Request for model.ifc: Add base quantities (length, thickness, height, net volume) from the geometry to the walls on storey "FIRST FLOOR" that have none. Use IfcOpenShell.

First a look at what the model holds.

```python
import ifcopenshell
import ifcopenshell.util.element
import ifcopenshell.util.unit

model = ifcopenshell.open("model.ifc")
print(model.schema)
for unit_type in ("LENGTHUNIT", "AREAUNIT", "VOLUMEUNIT"):
    print(unit_type, ifcopenshell.util.unit.calculate_unit_scale(model, unit_type))
storey = next(s for s in model.by_type("IfcBuildingStorey") if s.Name == "FIRST FLOOR")
walls = [e for e in ifcopenshell.util.element.get_decomposition(storey) if e.is_a("IfcWall")]
for e in sorted(walls, key=lambda e: e.id()):
    print(e.id(), e.is_a(), e.Name, list(ifcopenshell.util.element.get_psets(e, qtos_only=True)), sep=" | ")
```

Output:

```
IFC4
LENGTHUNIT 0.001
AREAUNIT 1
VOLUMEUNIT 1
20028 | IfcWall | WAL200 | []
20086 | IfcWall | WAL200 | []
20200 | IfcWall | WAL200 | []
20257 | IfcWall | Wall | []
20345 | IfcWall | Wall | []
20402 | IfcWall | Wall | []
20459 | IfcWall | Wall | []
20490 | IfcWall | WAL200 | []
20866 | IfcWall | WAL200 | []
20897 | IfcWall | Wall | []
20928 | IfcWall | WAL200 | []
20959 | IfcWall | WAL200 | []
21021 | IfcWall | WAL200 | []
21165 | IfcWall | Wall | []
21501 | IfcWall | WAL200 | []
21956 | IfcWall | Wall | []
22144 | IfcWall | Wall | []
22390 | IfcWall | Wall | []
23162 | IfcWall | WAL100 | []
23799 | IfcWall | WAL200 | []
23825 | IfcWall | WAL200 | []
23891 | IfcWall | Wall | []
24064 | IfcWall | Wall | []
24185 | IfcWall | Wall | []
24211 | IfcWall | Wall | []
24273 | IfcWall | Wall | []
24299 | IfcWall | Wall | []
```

```python
import ifcopenshell
import ifcopenshell.api.pset
import ifcopenshell.geom
import ifcopenshell.util.element
import ifcopenshell.util.shape
import ifcopenshell.util.unit

model = ifcopenshell.open("model.ifc")
unit_scale = ifcopenshell.util.unit.calculate_unit_scale(model)
volume_scale = ifcopenshell.util.unit.calculate_unit_scale(model, "VOLUMEUNIT")
settings = ifcopenshell.geom.settings()

storey = next(s for s in model.by_type("IfcBuildingStorey") if s.Name == "FIRST FLOOR")
walls = [e for e in ifcopenshell.util.element.get_decomposition(storey) if e.is_a("IfcWall")]

for e in sorted(walls, key=lambda e: e.id()):
    if ifcopenshell.util.element.get_psets(e, qtos_only=True, should_inherit=False):
        continue
    # Geometry comes back in metres, in the element's own axes.
    shape = ifcopenshell.geom.create_shape(settings, e)
    values = {
        "Length": ifcopenshell.util.shape.get_x(shape.geometry) / unit_scale,
        "Width": ifcopenshell.util.shape.get_y(shape.geometry) / unit_scale,
        "Height": ifcopenshell.util.shape.get_z(shape.geometry) / unit_scale,
        "NetVolume": ifcopenshell.util.shape.get_volume(shape.geometry) / volume_scale,
    }
    qto = ifcopenshell.api.pset.add_qto(model, product=e, name="Qto_WallBaseQuantities")
    ifcopenshell.api.pset.edit_qto(model, qto=qto, properties=values)
    print(e.id(), {k: round(v, 3) for k, v in values.items()})

model.write("model-out.ifc")
```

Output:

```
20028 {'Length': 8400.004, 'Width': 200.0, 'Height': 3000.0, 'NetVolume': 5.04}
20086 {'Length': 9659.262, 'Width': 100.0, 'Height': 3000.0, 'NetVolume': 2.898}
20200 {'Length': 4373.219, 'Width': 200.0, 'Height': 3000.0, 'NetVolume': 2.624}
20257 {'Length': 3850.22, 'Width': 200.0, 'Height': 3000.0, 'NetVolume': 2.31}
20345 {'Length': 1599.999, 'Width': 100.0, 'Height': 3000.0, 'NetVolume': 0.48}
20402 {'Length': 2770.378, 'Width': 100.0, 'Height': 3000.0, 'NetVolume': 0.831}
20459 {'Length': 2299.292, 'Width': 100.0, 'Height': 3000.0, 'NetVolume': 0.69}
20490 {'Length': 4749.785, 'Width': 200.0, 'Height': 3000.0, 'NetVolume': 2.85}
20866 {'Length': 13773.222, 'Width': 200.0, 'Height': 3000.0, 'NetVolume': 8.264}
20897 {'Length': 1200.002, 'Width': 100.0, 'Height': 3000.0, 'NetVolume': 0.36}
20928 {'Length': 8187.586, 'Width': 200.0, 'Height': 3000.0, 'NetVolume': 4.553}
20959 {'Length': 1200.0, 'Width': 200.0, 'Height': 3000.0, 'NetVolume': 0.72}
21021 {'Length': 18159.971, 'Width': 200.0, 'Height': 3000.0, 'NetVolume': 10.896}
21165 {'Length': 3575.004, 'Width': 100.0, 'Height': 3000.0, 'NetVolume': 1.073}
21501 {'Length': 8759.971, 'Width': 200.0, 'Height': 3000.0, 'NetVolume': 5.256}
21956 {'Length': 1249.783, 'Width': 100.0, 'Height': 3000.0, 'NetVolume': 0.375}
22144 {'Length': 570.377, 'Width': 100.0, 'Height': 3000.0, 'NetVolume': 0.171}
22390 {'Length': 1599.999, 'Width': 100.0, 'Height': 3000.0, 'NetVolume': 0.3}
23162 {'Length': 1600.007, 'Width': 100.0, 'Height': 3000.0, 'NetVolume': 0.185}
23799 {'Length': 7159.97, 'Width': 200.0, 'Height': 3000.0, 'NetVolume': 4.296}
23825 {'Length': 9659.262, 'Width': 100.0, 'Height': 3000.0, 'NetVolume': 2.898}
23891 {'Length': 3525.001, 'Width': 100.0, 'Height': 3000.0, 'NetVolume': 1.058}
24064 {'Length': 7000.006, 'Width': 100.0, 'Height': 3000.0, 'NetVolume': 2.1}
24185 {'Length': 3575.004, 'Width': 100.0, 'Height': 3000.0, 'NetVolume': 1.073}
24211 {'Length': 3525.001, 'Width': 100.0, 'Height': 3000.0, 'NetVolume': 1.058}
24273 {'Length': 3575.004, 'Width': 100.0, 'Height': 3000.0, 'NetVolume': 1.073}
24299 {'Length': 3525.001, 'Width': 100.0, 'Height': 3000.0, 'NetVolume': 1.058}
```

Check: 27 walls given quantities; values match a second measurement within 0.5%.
